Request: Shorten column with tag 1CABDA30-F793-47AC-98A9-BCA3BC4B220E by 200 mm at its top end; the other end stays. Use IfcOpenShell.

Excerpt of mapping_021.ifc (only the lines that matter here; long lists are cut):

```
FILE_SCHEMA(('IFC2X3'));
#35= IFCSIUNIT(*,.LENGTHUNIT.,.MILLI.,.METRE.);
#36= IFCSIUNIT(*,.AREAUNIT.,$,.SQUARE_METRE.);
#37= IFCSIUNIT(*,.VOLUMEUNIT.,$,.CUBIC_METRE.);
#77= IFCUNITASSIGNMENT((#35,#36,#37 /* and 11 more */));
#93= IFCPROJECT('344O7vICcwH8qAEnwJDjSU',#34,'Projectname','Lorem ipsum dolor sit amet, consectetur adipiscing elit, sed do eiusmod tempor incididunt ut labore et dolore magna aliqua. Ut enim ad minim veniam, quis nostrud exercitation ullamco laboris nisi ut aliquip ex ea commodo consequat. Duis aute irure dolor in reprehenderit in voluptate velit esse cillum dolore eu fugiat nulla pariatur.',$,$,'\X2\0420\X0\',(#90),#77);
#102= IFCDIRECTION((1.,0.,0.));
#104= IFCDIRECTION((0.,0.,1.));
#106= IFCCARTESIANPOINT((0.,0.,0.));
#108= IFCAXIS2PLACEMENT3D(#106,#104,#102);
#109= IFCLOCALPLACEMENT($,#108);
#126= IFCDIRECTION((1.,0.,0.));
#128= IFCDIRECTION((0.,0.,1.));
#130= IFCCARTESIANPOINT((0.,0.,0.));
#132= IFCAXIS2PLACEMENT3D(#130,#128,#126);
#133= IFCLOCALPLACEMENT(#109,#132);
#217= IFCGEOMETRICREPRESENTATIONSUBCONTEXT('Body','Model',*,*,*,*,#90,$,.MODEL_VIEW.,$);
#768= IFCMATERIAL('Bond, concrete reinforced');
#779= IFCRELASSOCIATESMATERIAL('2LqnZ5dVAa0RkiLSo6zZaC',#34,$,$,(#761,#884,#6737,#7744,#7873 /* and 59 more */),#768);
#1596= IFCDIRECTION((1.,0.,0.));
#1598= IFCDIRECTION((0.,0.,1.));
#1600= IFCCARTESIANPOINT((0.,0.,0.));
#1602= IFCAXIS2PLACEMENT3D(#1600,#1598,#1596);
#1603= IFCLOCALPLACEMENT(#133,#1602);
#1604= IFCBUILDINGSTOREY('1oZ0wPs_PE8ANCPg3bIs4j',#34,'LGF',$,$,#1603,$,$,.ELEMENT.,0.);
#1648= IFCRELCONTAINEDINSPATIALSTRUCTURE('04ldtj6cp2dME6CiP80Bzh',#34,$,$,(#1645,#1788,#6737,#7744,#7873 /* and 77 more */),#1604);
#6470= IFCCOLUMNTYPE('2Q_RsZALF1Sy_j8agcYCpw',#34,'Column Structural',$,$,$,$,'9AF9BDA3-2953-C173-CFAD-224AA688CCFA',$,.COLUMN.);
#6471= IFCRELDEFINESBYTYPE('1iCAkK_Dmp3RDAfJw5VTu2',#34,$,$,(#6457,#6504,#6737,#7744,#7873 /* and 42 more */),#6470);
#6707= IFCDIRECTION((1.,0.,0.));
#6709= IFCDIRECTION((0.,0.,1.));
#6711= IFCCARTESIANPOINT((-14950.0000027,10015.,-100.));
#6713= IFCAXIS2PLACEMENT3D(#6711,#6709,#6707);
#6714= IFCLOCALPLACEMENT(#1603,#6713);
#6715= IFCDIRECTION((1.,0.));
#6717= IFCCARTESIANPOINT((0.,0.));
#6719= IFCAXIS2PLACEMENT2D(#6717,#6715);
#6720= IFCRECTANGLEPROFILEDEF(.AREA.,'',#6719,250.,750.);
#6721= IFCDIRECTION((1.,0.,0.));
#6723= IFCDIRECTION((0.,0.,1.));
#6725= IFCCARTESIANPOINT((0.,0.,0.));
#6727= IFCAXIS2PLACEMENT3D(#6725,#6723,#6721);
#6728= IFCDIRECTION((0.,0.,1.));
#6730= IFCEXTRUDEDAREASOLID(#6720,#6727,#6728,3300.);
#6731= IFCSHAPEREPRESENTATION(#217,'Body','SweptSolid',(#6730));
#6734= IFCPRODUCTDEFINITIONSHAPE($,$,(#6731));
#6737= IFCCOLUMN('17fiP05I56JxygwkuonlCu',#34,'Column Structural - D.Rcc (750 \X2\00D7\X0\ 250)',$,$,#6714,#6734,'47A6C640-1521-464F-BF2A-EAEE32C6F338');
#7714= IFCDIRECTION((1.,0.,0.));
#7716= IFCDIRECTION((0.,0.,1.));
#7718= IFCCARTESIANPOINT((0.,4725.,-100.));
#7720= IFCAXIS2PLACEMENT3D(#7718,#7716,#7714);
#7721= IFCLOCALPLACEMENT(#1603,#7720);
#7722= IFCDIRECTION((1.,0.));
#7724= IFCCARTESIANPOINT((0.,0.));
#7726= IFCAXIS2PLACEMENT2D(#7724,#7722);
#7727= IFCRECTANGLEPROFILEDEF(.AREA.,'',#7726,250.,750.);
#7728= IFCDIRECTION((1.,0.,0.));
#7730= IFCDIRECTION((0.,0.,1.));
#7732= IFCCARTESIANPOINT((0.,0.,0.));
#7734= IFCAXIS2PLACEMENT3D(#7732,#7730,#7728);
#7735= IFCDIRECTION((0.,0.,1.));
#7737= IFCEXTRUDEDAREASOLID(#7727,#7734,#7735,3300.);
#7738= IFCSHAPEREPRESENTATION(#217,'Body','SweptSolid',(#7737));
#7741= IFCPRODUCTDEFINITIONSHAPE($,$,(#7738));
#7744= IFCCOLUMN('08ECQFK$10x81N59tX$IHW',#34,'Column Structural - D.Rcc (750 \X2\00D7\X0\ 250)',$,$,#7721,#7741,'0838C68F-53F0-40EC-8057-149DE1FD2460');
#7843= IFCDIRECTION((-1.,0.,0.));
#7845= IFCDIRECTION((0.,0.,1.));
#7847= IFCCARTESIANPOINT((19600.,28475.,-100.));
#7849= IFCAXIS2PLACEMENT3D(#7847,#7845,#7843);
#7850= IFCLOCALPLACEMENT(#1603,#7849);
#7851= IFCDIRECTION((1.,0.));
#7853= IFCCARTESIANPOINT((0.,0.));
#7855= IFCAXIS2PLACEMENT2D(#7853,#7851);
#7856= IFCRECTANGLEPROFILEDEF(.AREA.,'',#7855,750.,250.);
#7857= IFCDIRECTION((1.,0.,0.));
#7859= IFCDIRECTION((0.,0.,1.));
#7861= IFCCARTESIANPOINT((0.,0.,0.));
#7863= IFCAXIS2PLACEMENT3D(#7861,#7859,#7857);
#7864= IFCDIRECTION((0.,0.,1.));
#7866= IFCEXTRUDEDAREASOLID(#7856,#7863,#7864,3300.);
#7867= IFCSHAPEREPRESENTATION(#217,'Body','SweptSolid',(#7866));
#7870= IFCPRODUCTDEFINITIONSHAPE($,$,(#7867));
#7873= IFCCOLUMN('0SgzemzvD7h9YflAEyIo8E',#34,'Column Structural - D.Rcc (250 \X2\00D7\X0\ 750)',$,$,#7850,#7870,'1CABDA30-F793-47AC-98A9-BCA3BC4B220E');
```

```python
import ifcopenshell
import ifcopenshell.util.representation
import ifcopenshell.util.unit

model = ifcopenshell.open("mapping_021.ifc")
unit_scale = ifcopenshell.util.unit.calculate_unit_scale(model)

member = model.by_id(7873)
change = -0.2 / unit_scale

# The extrusion runs towards the end named, so only its depth changes.
body = ifcopenshell.util.representation.get_representation(member, "Model", "Body")
solid = body.Items[0]
old_length = solid.Depth
solid.Depth += change

print(f"length {old_length:g} -> {solid.Depth:g}")

model.write("mapping_021_edited.ifc")
```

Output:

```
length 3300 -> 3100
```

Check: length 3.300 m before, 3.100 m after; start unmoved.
